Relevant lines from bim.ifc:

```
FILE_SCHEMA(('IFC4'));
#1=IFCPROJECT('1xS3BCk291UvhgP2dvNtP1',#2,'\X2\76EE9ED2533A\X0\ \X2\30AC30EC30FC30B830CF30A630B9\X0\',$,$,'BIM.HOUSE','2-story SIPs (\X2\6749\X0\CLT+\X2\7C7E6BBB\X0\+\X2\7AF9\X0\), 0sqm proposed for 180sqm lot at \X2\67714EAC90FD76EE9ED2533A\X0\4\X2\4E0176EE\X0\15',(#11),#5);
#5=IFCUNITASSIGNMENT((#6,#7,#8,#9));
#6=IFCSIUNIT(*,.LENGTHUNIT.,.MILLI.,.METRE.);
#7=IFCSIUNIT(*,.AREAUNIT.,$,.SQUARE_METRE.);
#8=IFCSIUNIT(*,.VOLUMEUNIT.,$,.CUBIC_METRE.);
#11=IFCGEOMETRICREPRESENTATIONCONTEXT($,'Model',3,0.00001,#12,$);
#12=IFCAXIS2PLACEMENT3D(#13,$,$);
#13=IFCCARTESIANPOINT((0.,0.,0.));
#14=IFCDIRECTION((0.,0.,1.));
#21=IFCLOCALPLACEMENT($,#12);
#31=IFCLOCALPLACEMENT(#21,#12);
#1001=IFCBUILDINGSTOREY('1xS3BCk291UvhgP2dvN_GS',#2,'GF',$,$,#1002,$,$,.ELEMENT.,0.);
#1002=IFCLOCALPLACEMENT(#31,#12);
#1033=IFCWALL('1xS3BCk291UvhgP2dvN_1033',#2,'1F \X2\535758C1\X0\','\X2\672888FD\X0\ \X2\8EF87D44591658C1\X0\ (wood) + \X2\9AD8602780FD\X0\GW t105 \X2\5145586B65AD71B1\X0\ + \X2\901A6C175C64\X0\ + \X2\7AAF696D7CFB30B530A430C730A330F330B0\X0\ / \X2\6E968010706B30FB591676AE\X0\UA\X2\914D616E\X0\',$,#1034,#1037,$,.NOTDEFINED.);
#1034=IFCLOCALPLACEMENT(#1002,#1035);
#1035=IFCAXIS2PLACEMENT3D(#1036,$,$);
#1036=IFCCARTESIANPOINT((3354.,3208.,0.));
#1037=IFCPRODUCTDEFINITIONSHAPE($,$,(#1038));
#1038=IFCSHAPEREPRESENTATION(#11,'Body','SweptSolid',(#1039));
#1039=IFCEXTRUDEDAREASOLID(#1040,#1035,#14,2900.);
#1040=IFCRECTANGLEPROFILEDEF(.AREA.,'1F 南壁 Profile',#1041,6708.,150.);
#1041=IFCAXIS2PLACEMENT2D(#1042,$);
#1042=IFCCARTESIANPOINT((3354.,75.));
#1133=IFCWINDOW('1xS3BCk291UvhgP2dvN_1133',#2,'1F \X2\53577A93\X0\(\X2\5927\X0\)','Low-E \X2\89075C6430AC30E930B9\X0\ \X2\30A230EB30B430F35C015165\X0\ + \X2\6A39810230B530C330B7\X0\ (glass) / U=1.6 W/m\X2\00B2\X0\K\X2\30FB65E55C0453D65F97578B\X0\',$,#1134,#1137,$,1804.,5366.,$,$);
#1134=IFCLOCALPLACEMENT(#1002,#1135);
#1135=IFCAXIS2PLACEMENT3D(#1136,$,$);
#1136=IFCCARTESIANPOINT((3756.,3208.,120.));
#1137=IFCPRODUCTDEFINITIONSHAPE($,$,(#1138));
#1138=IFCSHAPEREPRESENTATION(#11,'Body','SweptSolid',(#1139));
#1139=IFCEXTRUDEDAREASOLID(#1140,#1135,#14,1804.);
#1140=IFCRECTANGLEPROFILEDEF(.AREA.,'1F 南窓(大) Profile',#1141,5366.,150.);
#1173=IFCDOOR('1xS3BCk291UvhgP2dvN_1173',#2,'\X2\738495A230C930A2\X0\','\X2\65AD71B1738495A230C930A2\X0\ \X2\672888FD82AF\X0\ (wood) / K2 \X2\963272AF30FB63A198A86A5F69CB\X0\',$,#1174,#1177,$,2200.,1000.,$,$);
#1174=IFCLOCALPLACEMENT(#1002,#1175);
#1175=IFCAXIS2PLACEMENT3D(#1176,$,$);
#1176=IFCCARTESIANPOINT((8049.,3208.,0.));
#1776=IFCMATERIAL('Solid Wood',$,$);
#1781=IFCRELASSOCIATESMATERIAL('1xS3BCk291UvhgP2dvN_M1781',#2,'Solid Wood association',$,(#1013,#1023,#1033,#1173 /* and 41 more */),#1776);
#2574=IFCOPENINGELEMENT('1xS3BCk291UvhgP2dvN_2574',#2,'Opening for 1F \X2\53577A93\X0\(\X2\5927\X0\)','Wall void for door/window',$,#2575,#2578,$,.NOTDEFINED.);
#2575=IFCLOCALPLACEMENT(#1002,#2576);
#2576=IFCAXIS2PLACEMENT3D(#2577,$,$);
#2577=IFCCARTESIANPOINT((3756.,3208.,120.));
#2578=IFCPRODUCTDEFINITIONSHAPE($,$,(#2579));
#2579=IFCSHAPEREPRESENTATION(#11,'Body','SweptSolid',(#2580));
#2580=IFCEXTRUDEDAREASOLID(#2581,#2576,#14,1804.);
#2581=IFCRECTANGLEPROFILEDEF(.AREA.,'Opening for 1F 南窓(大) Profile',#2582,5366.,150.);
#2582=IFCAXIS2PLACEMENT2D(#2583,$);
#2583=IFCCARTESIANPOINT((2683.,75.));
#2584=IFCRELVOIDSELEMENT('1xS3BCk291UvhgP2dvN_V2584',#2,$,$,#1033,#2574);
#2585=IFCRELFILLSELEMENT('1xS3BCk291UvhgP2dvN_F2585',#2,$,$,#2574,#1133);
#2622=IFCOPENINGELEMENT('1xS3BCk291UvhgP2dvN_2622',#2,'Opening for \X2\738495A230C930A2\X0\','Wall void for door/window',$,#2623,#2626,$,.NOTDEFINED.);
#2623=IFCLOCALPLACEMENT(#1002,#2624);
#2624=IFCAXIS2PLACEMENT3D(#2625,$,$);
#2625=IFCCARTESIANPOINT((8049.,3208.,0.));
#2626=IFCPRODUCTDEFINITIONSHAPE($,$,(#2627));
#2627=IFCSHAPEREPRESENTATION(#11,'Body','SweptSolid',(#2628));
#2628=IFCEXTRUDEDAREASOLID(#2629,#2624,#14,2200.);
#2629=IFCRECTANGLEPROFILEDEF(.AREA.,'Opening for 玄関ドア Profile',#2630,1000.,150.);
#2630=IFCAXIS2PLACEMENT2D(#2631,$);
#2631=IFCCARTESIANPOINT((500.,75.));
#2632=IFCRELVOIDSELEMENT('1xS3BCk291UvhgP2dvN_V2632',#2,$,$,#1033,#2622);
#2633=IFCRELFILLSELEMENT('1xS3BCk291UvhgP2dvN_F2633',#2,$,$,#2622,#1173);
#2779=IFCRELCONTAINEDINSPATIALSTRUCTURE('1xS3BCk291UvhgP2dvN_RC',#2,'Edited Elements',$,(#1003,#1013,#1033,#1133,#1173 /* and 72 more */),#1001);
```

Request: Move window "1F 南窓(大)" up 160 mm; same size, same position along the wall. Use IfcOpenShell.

```python
import numpy as np
import ifcopenshell
import ifcopenshell.api.geometry
import ifcopenshell.util.placement
import ifcopenshell.util.unit

model = ifcopenshell.open("bim.ifc")
unit_scale = ifcopenshell.util.unit.calculate_unit_scale(model)

window = model.by_guid("1xS3BCk291UvhgP2dvN_1133")
opening = window.FillsVoids[0].RelatingOpeningElement
dz = 0.16 / unit_scale

shift = np.array([0.0, 0.0, dz])
# The window is not placed relative to its opening, so move both.
for product in (opening, window):
    matrix = ifcopenshell.util.placement.get_local_placement(product.ObjectPlacement)
    matrix[:3, 3] += shift
    ifcopenshell.api.geometry.edit_object_placement(model, product=product, matrix=matrix, is_si=False)

print(f"moved by {dz * unit_scale:+.3f} m")

model.write("bim_edited.ifc")
```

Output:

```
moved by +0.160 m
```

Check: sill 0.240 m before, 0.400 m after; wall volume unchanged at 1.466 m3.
